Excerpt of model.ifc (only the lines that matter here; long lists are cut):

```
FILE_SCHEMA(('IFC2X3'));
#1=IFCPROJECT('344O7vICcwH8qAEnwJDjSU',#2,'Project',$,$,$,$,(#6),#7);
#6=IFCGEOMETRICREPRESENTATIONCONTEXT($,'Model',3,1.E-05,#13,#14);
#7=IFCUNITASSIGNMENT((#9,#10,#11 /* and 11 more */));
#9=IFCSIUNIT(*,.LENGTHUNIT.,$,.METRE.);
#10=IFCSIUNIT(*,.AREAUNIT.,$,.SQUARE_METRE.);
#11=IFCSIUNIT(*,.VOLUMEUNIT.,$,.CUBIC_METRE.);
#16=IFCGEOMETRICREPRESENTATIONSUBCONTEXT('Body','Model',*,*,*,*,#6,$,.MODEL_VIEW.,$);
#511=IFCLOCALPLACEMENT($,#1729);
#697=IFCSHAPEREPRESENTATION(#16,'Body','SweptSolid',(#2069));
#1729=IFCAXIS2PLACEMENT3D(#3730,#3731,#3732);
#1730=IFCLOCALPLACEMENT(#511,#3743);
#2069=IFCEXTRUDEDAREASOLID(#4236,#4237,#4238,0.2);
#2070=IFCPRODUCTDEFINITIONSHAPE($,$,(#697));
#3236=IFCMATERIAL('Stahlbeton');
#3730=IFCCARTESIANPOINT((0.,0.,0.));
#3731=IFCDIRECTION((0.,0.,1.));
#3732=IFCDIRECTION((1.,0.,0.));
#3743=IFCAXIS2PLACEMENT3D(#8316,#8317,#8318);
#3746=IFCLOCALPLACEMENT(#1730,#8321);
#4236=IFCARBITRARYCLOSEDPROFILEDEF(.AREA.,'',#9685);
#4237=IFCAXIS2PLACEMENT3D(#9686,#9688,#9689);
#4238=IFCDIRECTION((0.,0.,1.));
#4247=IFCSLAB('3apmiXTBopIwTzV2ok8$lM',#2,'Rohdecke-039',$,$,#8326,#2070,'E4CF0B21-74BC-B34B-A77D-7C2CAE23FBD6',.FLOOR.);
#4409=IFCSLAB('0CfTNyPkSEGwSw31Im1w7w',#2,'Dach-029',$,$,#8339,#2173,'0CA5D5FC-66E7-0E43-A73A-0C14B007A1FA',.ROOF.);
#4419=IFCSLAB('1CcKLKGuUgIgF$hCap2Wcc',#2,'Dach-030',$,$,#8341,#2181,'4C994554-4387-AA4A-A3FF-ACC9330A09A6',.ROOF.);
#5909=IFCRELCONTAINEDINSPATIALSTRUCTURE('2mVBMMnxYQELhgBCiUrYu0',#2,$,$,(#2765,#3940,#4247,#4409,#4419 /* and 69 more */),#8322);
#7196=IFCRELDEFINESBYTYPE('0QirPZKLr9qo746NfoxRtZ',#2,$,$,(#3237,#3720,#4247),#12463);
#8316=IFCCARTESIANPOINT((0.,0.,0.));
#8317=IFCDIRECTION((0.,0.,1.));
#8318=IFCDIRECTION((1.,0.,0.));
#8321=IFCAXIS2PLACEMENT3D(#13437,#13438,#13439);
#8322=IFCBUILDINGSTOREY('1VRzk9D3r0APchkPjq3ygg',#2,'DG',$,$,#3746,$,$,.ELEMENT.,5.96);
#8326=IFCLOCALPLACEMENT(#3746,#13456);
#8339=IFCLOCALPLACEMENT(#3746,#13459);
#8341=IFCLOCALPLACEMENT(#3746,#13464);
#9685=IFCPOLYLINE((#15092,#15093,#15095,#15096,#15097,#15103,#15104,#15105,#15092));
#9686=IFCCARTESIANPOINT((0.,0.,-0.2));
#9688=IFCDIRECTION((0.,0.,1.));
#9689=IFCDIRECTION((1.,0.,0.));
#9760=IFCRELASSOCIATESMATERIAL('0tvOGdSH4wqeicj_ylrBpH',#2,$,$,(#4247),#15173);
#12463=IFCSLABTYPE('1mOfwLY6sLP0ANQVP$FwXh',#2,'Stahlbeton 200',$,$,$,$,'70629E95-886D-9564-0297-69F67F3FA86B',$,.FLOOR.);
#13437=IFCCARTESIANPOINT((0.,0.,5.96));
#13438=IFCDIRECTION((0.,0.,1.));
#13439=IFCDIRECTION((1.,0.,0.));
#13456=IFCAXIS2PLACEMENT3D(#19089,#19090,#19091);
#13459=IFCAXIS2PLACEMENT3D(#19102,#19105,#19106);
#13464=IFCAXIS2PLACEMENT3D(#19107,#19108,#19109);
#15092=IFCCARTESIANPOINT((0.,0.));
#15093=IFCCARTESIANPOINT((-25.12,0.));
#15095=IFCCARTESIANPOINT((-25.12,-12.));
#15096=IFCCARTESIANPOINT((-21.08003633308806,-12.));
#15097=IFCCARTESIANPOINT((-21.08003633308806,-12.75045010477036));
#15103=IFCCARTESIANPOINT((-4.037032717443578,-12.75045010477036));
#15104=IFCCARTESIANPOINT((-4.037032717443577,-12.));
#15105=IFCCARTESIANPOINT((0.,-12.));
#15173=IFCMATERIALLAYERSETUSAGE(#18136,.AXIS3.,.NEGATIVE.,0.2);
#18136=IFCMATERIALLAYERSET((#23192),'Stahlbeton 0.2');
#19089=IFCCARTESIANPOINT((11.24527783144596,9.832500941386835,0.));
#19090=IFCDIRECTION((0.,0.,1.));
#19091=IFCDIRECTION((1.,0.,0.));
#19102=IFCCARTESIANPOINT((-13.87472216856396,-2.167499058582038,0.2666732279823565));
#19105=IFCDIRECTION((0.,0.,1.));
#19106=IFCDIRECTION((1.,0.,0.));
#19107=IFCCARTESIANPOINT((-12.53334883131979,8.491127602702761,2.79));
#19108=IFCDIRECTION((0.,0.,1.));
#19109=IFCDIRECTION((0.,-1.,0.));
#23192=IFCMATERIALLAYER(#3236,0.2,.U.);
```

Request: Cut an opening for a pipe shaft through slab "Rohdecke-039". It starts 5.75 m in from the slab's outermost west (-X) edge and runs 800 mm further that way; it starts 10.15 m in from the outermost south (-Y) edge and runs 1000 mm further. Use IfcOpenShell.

```python
import numpy as np
import ifcopenshell
import ifcopenshell.api.feature
import ifcopenshell.api.geometry
import ifcopenshell.api.root
import ifcopenshell.geom
import ifcopenshell.util.placement
import ifcopenshell.util.representation
import ifcopenshell.util.shape
import ifcopenshell.util.unit

model = ifcopenshell.open("model.ifc")
unit_scale = ifcopenshell.util.unit.calculate_unit_scale(model)
settings = ifcopenshell.geom.settings()


def volume(element):
    """Net volume in cubic metres, openings subtracted."""
    shape = ifcopenshell.geom.create_shape(settings, element)
    return ifcopenshell.util.shape.get_volume(shape.geometry)


slab = model.by_guid("3apmiXTBopIwTzV2ok8$lM")
before = volume(slab)

# Extent in the slab's own axes, in metres. The edges named are its -X and -Y sides.
slab_shape = ifcopenshell.geom.create_shape(settings, slab)
vertices = ifcopenshell.util.shape.get_vertices(slab_shape.geometry)
x_min, y_min, bottom = vertices.min(axis=0)
top = vertices[:, 2].max()

opening = ifcopenshell.api.root.create_entity(model, ifc_class="IfcOpeningElement", name="Pipe shaft opening")
context = ifcopenshell.util.representation.get_context(model, "Model", "Body", "MODEL_VIEW")
width, depth = 0.8, 1
outline = [(0.0, 0.0), (width, 0.0), (width, depth), (0.0, depth), (0.0, 0.0)]
# Overshoot both faces by 50 mm so the cut is clean.
shape = ifcopenshell.api.geometry.add_slab_representation(
    model, context=context, depth=top - bottom + 0.1, polyline=outline
)
ifcopenshell.api.geometry.assign_representation(model, product=opening, representation=shape)

matrix = ifcopenshell.util.placement.get_local_placement(slab.ObjectPlacement)
matrix[:, 3] = matrix @ np.append(np.array([x_min + 5.75, y_min + 10.15, bottom - 0.05]) / unit_scale, 1.0)
ifcopenshell.api.geometry.edit_object_placement(model, product=opening, matrix=matrix, is_si=False)
ifcopenshell.api.feature.add_feature(model, feature=opening, element=slab)

after = volume(slab)

print(f"slab volume {before:.3f} -> {after:.3f} m3")

model.write("model_v2.ifc")
```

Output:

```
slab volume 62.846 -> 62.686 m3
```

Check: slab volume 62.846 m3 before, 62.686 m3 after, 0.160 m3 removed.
